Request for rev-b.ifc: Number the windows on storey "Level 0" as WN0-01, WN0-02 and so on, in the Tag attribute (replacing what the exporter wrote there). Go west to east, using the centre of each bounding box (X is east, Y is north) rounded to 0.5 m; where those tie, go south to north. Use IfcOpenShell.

First a look at what the model holds.

```python
import ifcopenshell
import ifcopenshell.util.element
import ifcopenshell.util.placement

model = ifcopenshell.open("rev-b.ifc")
print(model.schema)
storey = next(s for s in model.by_type("IfcBuildingStorey") if s.Name == "Level 0")
windows = [e for e in ifcopenshell.util.element.get_decomposition(storey) if e.is_a("IfcWindow")]
for e in sorted(windows, key=lambda e: e.id()):
    origin = ifcopenshell.util.placement.get_local_placement(e.ObjectPlacement)[:3, 3]
    print(e.id(), e.Tag, e.Name, origin.round(2) + 0.0, sep=" | ")
```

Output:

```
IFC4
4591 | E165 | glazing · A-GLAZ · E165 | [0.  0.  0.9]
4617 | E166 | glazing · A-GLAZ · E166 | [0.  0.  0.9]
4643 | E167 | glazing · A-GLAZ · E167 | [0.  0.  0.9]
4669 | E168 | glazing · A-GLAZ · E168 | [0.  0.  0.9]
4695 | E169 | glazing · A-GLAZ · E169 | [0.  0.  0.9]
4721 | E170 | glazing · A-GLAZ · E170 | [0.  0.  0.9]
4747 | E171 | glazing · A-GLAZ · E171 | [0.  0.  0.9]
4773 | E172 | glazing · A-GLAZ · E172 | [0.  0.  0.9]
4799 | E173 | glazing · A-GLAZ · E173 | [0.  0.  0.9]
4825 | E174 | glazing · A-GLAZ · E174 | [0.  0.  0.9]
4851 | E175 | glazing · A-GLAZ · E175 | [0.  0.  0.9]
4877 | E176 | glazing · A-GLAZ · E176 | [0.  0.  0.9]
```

```python
import ifcopenshell
import ifcopenshell.geom
import ifcopenshell.util.element
import ifcopenshell.util.shape

model = ifcopenshell.open("rev-b.ifc")
settings = ifcopenshell.geom.settings()
settings.set("use-world-coords", True)


def centre(element):
    shape = ifcopenshell.geom.create_shape(settings, element)
    return ifcopenshell.util.shape.get_bbox_centroid(shape.geometry)


storey = next(s for s in model.by_type("IfcBuildingStorey") if s.Name == "Level 0")
windows = [e for e in ifcopenshell.util.element.get_decomposition(storey) if e.is_a("IfcWindow")]

# Insertion points can sit at a corner or the storey origin, so sort by the geometry (in metres).
centres = {e: centre(e) for e in windows}
windows.sort(key=lambda e: (round(centres[e][0] / 0.5), centres[e][1]))

for i, e in enumerate(windows, start=1):
    number = f"WN0-{i:02d}"
    e.Tag = number
    print(e.id(), number)

model.write("rev-b_updated.ifc")
```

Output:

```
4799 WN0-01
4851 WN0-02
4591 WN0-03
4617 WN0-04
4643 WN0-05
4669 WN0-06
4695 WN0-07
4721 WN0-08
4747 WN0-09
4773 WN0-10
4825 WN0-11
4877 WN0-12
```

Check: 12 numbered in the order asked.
